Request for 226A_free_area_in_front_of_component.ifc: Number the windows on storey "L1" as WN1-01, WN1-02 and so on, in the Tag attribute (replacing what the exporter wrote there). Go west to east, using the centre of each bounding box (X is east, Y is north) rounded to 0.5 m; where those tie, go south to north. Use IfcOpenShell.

First a look at what the model holds.

```python
import ifcopenshell
import ifcopenshell.util.element
import ifcopenshell.util.placement

model = ifcopenshell.open("226A_free_area_in_front_of_component.ifc")
print(model.schema)
storey = next(s for s in model.by_type("IfcBuildingStorey") if s.Name == "L1")
windows = [e for e in ifcopenshell.util.element.get_decomposition(storey) if e.is_a("IfcWindow")]
for e in sorted(windows, key=lambda e: e.id()):
    origin = ifcopenshell.util.placement.get_local_placement(e.ObjectPlacement)[:3, 3]
    print(e.id(), e.Tag, e.Name, origin.round(2) + 0.0, sep=" | ")
```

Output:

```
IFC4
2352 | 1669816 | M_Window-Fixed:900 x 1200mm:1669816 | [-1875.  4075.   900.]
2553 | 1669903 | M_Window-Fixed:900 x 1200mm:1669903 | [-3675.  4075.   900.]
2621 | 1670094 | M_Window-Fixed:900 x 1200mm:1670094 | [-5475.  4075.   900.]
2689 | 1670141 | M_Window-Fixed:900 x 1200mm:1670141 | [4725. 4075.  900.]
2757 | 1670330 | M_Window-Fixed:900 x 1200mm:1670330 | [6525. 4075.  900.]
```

```python
import ifcopenshell
import ifcopenshell.geom
import ifcopenshell.util.element
import ifcopenshell.util.shape

model = ifcopenshell.open("226A_free_area_in_front_of_component.ifc")
settings = ifcopenshell.geom.settings()
settings.set("use-world-coords", True)


def centre(element):
    shape = ifcopenshell.geom.create_shape(settings, element)
    return ifcopenshell.util.shape.get_bbox_centroid(shape.geometry)


storey = next(s for s in model.by_type("IfcBuildingStorey") if s.Name == "L1")
windows = [e for e in ifcopenshell.util.element.get_decomposition(storey) if e.is_a("IfcWindow")]

# Insertion points can sit at a corner or the storey origin, so sort by the geometry (in metres).
centres = {e: centre(e) for e in windows}
windows.sort(key=lambda e: (round(centres[e][0] / 0.5), centres[e][1]))

for i, e in enumerate(windows, start=1):
    number = f"WN1-{i:02d}"
    e.Tag = number
    print(e.id(), number)

model.write("226A_free_area_in_front_of_component_updated.ifc")
```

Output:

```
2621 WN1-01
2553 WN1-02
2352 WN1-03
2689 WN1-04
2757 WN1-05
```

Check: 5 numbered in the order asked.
